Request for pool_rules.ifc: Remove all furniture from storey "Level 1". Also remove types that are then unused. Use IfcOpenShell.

First a look at what the model holds.

```python
import ifcopenshell
import ifcopenshell.util.element

model = ifcopenshell.open("pool_rules.ifc")
print(model.schema)
storey = next(s for s in model.by_type("IfcBuildingStorey") if s.Name == "Level 1")
furniture = [e for e in ifcopenshell.util.element.get_decomposition(storey) if e.is_a("IfcFurnishingElement")]
seen = {}
for e in furniture:
    element_type = ifcopenshell.util.element.get_type(e)
    name = element_type.Name if element_type not in (None, e) else None
    seen[name] = seen.get(name, 0) + 1
for name, count in sorted(seen.items(), key=str):
    print(count, "x", name)
```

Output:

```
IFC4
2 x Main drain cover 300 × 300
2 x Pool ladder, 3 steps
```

```python
import ifcopenshell
import ifcopenshell.api.root
import ifcopenshell.util.element

model = ifcopenshell.open("pool_rules.ifc")

storey = next(s for s in model.by_type("IfcBuildingStorey") if s.Name == "Level 1")
furniture = [e for e in ifcopenshell.util.element.get_decomposition(storey) if e.is_a("IfcFurnishingElement")]
types = {ifcopenshell.util.element.get_type(e) for e in furniture} - {None, *furniture}

for e in furniture:
    ifcopenshell.api.root.remove_product(model, product=e)
print(len(furniture), "removed")

unused = [t for t in types if not ifcopenshell.util.element.get_types(t)]
for t in unused:
    ifcopenshell.api.root.remove_product(model, product=t)
print(len(unused), "unused types removed")

model.write("pool_rules_edited.ifc")
```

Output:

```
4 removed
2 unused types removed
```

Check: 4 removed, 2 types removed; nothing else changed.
